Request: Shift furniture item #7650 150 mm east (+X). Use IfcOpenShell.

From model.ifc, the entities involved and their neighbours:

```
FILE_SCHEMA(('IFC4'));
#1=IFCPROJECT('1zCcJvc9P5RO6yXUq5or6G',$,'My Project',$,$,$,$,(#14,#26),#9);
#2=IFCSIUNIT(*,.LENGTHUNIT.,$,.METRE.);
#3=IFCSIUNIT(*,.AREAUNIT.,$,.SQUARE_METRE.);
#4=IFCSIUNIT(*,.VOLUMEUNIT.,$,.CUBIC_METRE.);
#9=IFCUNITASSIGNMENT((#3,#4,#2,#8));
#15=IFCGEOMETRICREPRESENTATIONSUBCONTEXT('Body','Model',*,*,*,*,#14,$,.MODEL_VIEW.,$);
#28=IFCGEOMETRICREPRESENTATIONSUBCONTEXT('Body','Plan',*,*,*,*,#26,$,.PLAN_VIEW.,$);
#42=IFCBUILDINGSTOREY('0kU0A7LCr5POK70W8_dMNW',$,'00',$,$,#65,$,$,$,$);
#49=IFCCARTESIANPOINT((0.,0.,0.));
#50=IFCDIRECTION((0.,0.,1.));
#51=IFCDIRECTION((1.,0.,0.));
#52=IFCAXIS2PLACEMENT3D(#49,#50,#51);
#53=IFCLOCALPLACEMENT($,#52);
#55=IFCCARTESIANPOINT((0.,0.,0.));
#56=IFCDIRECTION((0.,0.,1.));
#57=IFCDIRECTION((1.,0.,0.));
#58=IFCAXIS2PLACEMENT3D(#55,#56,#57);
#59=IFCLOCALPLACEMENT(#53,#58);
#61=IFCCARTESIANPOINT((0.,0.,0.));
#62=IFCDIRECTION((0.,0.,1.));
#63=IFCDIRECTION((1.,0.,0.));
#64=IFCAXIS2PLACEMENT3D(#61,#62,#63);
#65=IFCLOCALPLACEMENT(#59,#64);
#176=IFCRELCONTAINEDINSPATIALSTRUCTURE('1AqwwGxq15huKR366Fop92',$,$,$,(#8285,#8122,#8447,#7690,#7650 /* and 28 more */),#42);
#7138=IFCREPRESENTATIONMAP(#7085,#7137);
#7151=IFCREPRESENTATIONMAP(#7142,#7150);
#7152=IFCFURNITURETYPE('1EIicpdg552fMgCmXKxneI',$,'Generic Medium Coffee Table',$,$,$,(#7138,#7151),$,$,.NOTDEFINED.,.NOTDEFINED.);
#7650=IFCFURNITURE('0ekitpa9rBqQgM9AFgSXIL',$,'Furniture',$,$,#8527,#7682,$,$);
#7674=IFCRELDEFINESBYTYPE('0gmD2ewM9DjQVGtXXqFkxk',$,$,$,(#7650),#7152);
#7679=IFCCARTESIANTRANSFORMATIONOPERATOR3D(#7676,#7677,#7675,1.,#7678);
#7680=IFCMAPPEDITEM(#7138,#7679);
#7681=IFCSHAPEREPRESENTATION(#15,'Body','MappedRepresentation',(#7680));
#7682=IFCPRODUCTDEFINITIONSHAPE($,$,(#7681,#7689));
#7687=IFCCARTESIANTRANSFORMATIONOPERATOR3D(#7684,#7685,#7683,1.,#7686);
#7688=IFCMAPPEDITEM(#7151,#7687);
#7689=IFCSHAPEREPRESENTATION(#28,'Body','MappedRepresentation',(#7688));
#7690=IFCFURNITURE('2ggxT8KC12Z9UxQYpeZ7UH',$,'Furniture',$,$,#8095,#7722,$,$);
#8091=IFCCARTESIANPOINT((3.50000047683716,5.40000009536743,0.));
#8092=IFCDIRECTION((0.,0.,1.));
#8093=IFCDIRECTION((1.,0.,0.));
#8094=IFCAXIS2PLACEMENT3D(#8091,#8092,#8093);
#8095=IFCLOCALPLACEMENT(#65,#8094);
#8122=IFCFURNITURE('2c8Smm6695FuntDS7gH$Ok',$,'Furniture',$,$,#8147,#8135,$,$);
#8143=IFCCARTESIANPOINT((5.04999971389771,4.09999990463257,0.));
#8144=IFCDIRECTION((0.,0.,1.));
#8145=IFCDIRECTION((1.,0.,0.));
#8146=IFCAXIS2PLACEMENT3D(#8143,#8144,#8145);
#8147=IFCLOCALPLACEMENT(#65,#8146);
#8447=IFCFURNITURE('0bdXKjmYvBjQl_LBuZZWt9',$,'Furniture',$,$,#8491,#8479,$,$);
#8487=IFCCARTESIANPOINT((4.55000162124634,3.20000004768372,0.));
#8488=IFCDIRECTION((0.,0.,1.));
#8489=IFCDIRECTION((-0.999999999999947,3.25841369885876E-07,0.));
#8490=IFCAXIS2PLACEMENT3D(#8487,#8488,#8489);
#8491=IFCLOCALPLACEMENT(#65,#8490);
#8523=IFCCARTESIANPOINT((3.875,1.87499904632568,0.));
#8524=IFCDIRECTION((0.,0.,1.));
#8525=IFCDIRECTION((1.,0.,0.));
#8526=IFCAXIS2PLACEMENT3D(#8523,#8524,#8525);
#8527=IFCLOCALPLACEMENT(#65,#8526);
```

```python
import ifcopenshell
import ifcopenshell.api.geometry
import ifcopenshell.util.placement

model = ifcopenshell.open("model.ifc")

item = model.by_id(7650)
matrix = ifcopenshell.util.placement.get_local_placement(item.ObjectPlacement)
matrix[0, 3] += 0.15
ifcopenshell.api.geometry.edit_object_placement(model, product=item, matrix=matrix, is_si=False)

print(ifcopenshell.util.placement.get_local_placement(item.ObjectPlacement).round(3) + 0.0)

model.write("model_rev.ifc")
```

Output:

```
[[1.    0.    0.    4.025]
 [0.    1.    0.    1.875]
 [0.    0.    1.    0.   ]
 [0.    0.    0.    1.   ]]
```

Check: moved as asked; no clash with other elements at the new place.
